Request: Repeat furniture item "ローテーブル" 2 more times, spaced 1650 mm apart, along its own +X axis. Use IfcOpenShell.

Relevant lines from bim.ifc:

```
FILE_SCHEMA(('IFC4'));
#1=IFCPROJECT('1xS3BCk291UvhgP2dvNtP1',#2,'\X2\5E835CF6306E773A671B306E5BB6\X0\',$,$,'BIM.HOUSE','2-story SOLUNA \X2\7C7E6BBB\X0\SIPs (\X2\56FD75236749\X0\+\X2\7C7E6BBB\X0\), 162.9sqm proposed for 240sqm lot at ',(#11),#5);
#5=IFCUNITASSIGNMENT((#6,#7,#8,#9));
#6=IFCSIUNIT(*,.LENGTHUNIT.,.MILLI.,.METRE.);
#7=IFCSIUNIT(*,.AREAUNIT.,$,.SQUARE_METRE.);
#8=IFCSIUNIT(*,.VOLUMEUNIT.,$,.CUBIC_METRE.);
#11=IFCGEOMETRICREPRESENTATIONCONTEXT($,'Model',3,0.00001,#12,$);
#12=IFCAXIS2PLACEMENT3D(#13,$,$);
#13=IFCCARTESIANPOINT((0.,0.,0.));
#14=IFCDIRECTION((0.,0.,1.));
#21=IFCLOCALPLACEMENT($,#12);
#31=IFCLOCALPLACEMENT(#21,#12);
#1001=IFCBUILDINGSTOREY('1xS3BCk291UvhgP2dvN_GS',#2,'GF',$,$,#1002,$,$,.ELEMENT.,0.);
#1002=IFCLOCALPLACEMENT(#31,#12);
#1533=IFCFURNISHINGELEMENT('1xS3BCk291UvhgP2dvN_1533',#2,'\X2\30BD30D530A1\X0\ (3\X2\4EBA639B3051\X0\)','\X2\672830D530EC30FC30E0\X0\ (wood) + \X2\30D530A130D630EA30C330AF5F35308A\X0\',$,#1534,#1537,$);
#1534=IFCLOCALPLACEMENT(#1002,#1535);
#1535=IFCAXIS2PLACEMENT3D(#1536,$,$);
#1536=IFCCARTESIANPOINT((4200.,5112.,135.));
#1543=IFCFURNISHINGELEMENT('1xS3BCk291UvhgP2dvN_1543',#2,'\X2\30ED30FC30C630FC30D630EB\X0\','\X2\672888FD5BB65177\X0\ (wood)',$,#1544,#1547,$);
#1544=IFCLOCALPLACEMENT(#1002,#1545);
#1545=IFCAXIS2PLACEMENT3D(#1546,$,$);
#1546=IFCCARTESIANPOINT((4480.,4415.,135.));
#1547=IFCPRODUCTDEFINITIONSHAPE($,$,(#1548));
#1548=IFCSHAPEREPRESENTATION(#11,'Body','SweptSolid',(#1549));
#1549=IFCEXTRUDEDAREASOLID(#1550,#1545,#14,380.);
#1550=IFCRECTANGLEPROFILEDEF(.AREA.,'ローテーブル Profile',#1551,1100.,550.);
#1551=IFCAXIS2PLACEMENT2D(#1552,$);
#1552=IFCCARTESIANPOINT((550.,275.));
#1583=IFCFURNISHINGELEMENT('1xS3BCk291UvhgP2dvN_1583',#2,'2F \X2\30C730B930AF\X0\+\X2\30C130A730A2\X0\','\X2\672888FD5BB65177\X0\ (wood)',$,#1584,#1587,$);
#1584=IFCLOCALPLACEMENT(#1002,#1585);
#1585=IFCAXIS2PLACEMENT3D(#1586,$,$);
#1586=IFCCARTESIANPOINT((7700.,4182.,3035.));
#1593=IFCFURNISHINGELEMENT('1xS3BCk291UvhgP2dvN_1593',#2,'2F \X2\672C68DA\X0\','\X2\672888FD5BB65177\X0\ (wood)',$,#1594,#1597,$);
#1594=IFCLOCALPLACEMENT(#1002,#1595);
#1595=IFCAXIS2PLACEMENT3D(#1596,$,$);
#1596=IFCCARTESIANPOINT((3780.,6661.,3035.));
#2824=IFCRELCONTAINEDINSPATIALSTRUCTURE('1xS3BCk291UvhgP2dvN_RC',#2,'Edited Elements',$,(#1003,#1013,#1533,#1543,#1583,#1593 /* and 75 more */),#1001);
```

```python
import ifcopenshell
import ifcopenshell.api.geometry
import ifcopenshell.api.root
import ifcopenshell.util.element
import ifcopenshell.util.placement

model = ifcopenshell.open("bim.ifc")


def reuse_history(source, copy):
    """copy_class also copies each property set's owner history, people and application; keep the originals."""
    for rel in copy.IsDefinedBy:
        if rel.is_a("IfcRelDefinesByProperties") and (history := rel.RelatingPropertyDefinition.OwnerHistory):
            rel.RelatingPropertyDefinition.OwnerHistory = source.OwnerHistory
            ifcopenshell.util.element.remove_deep2(model, history)


source = model.by_id(1543)
base = ifcopenshell.util.placement.get_local_placement(source.ObjectPlacement)
step = base[:3, 0] * 1650.0

for i in range(1, 3):
    copy = ifcopenshell.api.root.copy_class(model, product=source)
    copy.Representation = ifcopenshell.util.element.copy_deep(
        model, source.Representation, exclude=["IfcGeometricRepresentationContext", "IfcRepresentationMap"]
    )
    reuse_history(source, copy)
    matrix = base.copy()
    matrix[:3, 3] += i * step
    print("added at", matrix[:3, 3].round(3) + 0.0)
    ifcopenshell.api.geometry.edit_object_placement(model, product=copy, matrix=matrix, is_si=False)

model.write("bim-out.ifc")
```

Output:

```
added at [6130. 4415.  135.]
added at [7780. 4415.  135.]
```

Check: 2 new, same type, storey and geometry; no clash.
